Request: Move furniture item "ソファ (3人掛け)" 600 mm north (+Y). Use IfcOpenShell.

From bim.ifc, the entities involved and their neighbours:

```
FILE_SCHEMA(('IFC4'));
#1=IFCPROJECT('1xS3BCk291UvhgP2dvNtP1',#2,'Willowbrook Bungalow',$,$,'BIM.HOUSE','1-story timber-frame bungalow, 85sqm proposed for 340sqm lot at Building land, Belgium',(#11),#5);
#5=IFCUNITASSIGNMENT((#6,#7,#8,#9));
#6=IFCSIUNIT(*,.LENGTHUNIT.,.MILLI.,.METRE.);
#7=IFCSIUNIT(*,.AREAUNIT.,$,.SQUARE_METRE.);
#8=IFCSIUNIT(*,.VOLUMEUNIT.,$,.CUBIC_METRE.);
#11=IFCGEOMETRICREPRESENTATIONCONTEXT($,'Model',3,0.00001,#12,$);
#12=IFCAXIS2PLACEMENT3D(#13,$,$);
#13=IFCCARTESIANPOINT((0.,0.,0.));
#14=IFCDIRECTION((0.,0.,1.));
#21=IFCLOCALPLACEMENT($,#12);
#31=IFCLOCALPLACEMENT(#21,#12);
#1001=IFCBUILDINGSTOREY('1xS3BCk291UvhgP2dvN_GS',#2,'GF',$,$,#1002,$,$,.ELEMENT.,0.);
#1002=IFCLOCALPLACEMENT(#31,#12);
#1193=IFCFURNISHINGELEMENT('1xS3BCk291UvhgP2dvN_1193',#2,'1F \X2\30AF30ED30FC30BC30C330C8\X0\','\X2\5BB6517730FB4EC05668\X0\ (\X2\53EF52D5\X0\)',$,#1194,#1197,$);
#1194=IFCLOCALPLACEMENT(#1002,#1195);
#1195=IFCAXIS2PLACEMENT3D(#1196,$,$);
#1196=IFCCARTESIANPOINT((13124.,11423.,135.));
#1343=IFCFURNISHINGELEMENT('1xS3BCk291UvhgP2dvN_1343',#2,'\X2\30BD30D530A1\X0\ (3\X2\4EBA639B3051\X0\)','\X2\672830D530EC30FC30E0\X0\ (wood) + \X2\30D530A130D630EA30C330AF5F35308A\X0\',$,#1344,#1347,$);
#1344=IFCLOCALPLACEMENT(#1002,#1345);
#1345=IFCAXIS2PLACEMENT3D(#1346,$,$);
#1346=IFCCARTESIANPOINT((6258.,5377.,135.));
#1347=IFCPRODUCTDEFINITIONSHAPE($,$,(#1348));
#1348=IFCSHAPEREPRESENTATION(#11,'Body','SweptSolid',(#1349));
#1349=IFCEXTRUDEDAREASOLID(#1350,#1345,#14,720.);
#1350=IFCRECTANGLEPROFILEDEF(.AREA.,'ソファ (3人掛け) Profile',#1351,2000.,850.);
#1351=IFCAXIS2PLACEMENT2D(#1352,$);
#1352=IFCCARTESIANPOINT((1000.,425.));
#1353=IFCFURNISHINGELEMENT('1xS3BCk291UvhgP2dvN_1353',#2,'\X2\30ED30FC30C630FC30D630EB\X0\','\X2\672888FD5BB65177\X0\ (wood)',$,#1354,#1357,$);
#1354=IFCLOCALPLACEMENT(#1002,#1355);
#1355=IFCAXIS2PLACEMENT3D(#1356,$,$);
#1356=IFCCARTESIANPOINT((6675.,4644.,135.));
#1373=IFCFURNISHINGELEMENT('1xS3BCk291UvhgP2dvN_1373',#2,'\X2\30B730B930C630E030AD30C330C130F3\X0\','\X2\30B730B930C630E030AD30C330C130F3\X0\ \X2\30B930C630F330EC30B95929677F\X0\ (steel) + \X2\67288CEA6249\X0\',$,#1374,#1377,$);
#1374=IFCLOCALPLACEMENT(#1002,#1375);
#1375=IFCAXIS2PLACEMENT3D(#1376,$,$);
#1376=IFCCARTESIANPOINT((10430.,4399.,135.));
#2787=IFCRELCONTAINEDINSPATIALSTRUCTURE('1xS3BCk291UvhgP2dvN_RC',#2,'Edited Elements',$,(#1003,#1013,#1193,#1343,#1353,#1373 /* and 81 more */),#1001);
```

```python
import ifcopenshell
import ifcopenshell.api.geometry
import ifcopenshell.util.placement
import ifcopenshell.util.unit

model = ifcopenshell.open("bim.ifc")
unit_scale = ifcopenshell.util.unit.calculate_unit_scale(model)

item = model.by_guid("1xS3BCk291UvhgP2dvN_1343")
matrix = ifcopenshell.util.placement.get_local_placement(item.ObjectPlacement)
matrix[1, 3] += 0.6 / unit_scale
ifcopenshell.api.geometry.edit_object_placement(model, product=item, matrix=matrix, is_si=False)

print(ifcopenshell.util.placement.get_local_placement(item.ObjectPlacement).round(3) + 0.0)

model.write("bim-out.ifc")
```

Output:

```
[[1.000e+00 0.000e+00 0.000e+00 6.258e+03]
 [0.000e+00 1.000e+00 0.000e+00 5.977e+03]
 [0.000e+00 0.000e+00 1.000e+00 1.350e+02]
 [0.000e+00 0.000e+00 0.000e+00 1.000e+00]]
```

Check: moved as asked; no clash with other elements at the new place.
